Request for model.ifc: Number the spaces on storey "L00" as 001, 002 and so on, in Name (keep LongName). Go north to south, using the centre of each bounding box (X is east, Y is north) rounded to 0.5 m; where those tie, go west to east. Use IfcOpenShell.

First a look at what the model holds.

```python
import ifcopenshell
import ifcopenshell.util.element
import ifcopenshell.util.placement

model = ifcopenshell.open("model.ifc")
print(model.schema)
storey = next(s for s in model.by_type("IfcBuildingStorey") if s.Name == "L00")
spaces = [e for e in ifcopenshell.util.element.get_decomposition(storey) if e.is_a("IfcSpace")]
for e in sorted(spaces, key=lambda e: e.id()):
    origin = ifcopenshell.util.placement.get_local_placement(e.ObjectPlacement)[:3, 3]
    print(e.id(), e.Name, e.LongName, origin.round(2) + 0.0, sep=" | ")
```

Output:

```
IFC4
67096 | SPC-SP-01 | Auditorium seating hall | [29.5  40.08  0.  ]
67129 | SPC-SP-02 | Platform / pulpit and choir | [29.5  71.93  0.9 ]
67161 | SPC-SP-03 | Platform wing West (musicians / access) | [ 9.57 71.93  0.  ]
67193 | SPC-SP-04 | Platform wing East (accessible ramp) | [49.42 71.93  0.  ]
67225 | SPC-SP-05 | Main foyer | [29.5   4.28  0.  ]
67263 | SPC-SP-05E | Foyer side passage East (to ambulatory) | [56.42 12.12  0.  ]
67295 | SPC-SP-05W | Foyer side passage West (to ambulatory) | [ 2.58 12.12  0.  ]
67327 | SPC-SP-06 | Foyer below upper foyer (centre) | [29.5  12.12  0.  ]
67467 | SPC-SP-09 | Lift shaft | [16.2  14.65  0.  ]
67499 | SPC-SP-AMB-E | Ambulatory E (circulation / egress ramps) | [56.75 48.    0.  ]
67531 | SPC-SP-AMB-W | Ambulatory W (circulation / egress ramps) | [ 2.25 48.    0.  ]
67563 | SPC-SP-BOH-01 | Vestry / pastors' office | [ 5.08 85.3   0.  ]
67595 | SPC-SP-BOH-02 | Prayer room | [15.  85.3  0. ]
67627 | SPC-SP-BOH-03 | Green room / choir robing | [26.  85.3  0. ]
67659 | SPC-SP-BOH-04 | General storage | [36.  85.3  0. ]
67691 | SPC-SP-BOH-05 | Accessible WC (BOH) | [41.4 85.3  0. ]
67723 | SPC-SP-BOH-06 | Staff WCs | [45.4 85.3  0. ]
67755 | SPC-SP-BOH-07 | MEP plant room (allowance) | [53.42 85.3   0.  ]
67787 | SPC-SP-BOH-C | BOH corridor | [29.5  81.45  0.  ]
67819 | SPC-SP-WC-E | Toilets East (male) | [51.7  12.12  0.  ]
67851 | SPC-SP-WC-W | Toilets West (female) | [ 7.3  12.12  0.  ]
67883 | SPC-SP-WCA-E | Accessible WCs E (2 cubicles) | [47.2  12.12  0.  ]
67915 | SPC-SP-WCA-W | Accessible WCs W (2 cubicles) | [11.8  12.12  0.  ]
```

```python
import ifcopenshell
import ifcopenshell.geom
import ifcopenshell.util.element
import ifcopenshell.util.shape

model = ifcopenshell.open("model.ifc")
settings = ifcopenshell.geom.settings()
settings.set("use-world-coords", True)


def centre(element):
    shape = ifcopenshell.geom.create_shape(settings, element)
    return ifcopenshell.util.shape.get_bbox_centroid(shape.geometry)


storey = next(s for s in model.by_type("IfcBuildingStorey") if s.Name == "L00")
spaces = [e for e in ifcopenshell.util.element.get_decomposition(storey) if e.is_a("IfcSpace")]

# Insertion points can sit at a corner or the storey origin, so sort by the geometry (in metres).
centres = {e: centre(e) for e in spaces}
spaces.sort(key=lambda e: (-round(centres[e][1] / 0.5), centres[e][0]))

for i, e in enumerate(spaces, start=1):
    number = f"0{i:02d}"
    e.Name = number
    print(e.id(), number)

model.write("model_edited.ifc")
```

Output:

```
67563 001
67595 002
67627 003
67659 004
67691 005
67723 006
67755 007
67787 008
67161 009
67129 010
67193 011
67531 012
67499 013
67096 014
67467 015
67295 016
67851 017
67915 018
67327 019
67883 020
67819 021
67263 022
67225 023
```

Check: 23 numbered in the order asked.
